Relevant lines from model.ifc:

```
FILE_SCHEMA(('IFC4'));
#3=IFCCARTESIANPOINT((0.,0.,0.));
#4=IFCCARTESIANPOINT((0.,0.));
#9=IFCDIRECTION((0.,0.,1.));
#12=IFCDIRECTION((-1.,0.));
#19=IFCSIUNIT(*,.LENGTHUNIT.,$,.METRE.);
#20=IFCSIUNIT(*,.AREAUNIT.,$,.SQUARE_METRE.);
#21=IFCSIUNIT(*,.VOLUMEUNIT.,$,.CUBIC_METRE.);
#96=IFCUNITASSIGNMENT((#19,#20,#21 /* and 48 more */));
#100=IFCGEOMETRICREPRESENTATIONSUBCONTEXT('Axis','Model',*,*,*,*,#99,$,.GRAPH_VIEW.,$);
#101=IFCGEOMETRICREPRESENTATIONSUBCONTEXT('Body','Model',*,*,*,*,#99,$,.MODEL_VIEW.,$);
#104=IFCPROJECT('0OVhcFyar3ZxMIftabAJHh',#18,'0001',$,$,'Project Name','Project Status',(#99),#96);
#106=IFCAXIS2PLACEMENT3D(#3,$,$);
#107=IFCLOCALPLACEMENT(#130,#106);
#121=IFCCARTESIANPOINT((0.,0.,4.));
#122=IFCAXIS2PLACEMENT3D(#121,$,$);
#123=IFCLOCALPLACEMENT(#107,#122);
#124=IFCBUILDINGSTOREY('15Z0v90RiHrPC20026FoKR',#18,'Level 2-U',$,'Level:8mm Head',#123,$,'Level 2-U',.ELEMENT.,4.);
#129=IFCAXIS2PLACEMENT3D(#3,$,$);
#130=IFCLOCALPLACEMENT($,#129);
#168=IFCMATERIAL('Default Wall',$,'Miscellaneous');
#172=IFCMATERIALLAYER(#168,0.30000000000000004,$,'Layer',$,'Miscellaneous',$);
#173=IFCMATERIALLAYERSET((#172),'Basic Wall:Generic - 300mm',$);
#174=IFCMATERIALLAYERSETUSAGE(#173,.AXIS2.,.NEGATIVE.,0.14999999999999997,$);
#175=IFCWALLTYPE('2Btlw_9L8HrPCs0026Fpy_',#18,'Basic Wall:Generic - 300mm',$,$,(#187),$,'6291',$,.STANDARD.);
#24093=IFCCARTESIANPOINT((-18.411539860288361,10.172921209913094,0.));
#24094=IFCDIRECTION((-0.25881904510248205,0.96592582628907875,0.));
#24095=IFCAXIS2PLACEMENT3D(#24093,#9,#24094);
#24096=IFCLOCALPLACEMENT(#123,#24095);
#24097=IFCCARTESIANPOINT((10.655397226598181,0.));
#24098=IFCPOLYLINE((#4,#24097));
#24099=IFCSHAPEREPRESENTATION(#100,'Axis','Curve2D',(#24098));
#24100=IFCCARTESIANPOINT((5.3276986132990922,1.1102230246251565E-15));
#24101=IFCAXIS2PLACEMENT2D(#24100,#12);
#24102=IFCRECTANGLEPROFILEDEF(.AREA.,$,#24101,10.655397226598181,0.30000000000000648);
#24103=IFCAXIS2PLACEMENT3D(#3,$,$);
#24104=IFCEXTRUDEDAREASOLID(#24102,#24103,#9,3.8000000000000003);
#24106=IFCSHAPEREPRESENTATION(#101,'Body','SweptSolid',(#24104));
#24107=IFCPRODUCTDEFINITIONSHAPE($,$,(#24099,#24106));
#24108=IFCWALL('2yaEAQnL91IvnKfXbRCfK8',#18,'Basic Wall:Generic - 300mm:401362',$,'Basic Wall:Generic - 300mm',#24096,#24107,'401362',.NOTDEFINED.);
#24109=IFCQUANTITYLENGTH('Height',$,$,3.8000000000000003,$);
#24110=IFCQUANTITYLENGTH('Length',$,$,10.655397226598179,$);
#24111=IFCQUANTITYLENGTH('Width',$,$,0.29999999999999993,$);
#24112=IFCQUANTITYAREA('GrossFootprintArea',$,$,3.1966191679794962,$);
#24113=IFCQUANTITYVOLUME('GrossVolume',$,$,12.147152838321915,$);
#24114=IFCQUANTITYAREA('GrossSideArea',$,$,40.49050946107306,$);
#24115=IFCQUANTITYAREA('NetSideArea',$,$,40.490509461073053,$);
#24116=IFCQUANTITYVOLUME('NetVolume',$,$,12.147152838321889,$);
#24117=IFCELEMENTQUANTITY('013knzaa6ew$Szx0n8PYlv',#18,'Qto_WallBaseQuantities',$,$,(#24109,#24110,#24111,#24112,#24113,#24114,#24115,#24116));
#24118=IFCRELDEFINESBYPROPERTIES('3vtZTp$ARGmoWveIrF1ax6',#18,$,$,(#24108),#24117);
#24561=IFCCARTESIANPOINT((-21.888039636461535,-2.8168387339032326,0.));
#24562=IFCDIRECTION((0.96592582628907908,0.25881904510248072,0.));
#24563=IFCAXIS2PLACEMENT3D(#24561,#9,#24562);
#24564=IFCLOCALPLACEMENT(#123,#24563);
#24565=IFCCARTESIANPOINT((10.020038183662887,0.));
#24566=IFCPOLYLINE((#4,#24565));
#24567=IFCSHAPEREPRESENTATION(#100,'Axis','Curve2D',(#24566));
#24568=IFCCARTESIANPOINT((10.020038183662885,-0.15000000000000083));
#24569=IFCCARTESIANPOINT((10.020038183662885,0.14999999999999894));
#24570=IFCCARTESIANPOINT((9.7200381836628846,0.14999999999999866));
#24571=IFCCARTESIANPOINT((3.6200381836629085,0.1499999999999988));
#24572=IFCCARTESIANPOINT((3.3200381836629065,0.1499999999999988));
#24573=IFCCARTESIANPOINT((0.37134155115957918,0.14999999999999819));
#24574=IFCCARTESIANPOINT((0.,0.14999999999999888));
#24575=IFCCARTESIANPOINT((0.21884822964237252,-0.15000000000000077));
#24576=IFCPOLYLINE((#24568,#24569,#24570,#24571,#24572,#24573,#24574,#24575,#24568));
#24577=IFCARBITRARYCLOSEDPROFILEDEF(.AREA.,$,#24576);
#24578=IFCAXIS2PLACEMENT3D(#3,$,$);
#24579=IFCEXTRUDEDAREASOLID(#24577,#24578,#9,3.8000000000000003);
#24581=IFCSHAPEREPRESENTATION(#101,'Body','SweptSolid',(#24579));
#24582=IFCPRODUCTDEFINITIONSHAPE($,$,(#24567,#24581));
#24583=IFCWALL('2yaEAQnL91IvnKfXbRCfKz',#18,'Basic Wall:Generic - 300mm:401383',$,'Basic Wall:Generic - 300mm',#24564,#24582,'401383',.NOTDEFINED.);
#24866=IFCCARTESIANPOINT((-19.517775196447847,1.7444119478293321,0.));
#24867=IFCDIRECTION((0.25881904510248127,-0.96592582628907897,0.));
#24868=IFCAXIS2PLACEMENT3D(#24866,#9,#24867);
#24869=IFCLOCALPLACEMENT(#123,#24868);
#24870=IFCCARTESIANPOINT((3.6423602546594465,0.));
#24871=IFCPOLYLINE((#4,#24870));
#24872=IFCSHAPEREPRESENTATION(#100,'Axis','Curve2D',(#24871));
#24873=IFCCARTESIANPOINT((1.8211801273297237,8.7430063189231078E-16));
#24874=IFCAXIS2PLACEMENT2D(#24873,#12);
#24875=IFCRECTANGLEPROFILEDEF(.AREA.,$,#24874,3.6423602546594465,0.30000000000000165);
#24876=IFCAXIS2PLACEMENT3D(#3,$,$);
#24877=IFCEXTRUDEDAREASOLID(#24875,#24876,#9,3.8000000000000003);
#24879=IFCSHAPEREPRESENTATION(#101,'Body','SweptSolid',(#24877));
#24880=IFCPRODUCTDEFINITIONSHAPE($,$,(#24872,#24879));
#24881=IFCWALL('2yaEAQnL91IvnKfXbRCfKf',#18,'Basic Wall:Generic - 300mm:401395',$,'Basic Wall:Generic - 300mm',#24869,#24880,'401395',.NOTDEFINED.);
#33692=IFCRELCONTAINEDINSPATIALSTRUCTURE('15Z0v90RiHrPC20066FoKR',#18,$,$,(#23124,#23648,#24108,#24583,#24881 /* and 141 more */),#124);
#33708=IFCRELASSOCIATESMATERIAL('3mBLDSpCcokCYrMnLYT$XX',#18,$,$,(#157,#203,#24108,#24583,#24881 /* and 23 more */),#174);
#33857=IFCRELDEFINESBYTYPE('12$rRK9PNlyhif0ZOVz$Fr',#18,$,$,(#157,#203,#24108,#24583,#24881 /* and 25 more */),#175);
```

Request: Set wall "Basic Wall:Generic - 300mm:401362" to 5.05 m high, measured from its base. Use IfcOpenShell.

```python
import ifcopenshell
import ifcopenshell.api.pset
import ifcopenshell.geom
import ifcopenshell.util.element
import ifcopenshell.util.representation
import ifcopenshell.util.shape
import ifcopenshell.util.unit

model = ifcopenshell.open("model.ifc")
unit_scale = ifcopenshell.util.unit.calculate_unit_scale(model)
area_scale = ifcopenshell.util.unit.calculate_unit_scale(model, "AREAUNIT")
volume_scale = ifcopenshell.util.unit.calculate_unit_scale(model, "VOLUMEUNIT")
settings = ifcopenshell.geom.settings()


def volume(element):
    """Net volume in cubic metres, openings subtracted."""
    shape = ifcopenshell.geom.create_shape(settings, element)
    return ifcopenshell.util.shape.get_volume(shape.geometry)


wall = model.by_id(24108)
before = volume(wall)

body = ifcopenshell.util.representation.get_representation(wall, "Model", "Body")
solid = body.Items[0]
old_height = solid.Depth
solid.Depth = 5.05 / unit_scale
after = volume(wall)
thickness = 0.3  # wall thickness in metres

# Update the stored height, areas and volumes.
qto = model.by_id(ifcopenshell.util.element.get_pset(wall, "Qto_WallBaseQuantities", should_inherit=False)["id"])
ifcopenshell.api.pset.edit_qto(model, qto=qto, properties={
    "Height": solid.Depth,
    "GrossVolume": ifcopenshell.util.element.get_pset(wall, "Qto_WallBaseQuantities", "GrossVolume") * solid.Depth / old_height,
    "GrossSideArea": ifcopenshell.util.element.get_pset(wall, "Qto_WallBaseQuantities", "GrossSideArea") * solid.Depth / old_height,
    "NetSideArea": after / thickness / area_scale,
    "NetVolume": after / volume_scale,
})

print(f"height {old_height:g} -> {solid.Depth:g}, volume {before:.3f} -> {after:.3f} m3")

model.write("model_updated.ifc")
```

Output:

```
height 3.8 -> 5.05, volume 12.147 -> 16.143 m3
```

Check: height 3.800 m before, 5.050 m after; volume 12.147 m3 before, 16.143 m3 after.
